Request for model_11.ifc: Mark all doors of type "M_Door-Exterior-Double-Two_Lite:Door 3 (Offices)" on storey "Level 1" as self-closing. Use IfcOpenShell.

First a look at what the model holds.

```python
import ifcopenshell
import ifcopenshell.util.element

model = ifcopenshell.open("model_11.ifc")
print(model.schema)
storey = next(s for s in model.by_type("IfcBuildingStorey") if s.Name == "Level 1")
doors = [e for e in ifcopenshell.util.element.get_decomposition(storey) if e.is_a("IfcDoor")]
seen = {}
for e in doors:
    element_type = ifcopenshell.util.element.get_type(e)
    key = (element_type.Name if element_type != e and element_type else None, ifcopenshell.util.element.get_pset(e, "Pset_DoorCommon", "SelfClosing"))
    seen[key] = seen.get(key, 0) + 1
for (name, value), count in sorted(seen.items(), key=str):
    print(count, "x", name, "|", value)
```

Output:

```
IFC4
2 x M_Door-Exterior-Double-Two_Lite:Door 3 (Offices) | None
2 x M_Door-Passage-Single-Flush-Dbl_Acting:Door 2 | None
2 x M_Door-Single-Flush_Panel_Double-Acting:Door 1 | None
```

```python
import ifcopenshell
import ifcopenshell.api.pset
import ifcopenshell.util.element

model = ifcopenshell.open("model_11.ifc")

storey = next(s for s in model.by_type("IfcBuildingStorey") if s.Name == "Level 1")
doors = [e for e in ifcopenshell.util.element.get_decomposition(storey) if e.is_a("IfcDoor")]

count = 0
for e in doors:
    element_type = ifcopenshell.util.element.get_type(e)
    if element_type in (None, e) or element_type.Name != "M_Door-Exterior-Double-Two_Lite:Door 3 (Offices)":
        continue
    # add_pset returns the element's existing set when there is one.
    pset = ifcopenshell.api.pset.add_pset(model, product=e, name="Pset_DoorCommon")
    ifcopenshell.api.pset.edit_pset(model, pset=pset, properties={"SelfClosing": True})
    count += 1

print(count, "doors updated")

model.write("model_11_v2.ifc")
```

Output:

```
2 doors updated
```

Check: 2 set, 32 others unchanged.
